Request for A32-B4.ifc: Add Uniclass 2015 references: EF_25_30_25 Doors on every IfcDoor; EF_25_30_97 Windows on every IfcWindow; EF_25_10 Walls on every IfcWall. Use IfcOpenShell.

First a look at what the model holds.

```python
import ifcopenshell

model = ifcopenshell.open("A32-B4.ifc")
print(model.schema)
print("classifications:", [c.Name for c in model.by_type("IfcClassification")])
for ifc_class in ("IfcDoor", "IfcRoof", "IfcStair", "IfcWall", "IfcWindow"):
    print(ifc_class, len(model.by_type(ifc_class)))
```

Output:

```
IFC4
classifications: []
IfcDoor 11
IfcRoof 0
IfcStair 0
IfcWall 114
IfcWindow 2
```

```python
import ifcopenshell
import ifcopenshell.api.classification

model = ifcopenshell.open("A32-B4.ifc")

system = ifcopenshell.api.classification.add_classification(model, classification="Uniclass 2015")

codes = {
    "IfcDoor": ("EF_25_30_25", "Doors"),
    "IfcWindow": ("EF_25_30_97", "Windows"),
    "IfcWall": ("EF_25_10", "Walls"),
}
for ifc_class, (code, name) in codes.items():
    products = model.by_type(ifc_class)
    ifcopenshell.api.classification.add_reference(
        model, products=products, classification=system, identification=code, name=name
    )
    print(code, len(products))

model.write("A32-B4-out.ifc")
```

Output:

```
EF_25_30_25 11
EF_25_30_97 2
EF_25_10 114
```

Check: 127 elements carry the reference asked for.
